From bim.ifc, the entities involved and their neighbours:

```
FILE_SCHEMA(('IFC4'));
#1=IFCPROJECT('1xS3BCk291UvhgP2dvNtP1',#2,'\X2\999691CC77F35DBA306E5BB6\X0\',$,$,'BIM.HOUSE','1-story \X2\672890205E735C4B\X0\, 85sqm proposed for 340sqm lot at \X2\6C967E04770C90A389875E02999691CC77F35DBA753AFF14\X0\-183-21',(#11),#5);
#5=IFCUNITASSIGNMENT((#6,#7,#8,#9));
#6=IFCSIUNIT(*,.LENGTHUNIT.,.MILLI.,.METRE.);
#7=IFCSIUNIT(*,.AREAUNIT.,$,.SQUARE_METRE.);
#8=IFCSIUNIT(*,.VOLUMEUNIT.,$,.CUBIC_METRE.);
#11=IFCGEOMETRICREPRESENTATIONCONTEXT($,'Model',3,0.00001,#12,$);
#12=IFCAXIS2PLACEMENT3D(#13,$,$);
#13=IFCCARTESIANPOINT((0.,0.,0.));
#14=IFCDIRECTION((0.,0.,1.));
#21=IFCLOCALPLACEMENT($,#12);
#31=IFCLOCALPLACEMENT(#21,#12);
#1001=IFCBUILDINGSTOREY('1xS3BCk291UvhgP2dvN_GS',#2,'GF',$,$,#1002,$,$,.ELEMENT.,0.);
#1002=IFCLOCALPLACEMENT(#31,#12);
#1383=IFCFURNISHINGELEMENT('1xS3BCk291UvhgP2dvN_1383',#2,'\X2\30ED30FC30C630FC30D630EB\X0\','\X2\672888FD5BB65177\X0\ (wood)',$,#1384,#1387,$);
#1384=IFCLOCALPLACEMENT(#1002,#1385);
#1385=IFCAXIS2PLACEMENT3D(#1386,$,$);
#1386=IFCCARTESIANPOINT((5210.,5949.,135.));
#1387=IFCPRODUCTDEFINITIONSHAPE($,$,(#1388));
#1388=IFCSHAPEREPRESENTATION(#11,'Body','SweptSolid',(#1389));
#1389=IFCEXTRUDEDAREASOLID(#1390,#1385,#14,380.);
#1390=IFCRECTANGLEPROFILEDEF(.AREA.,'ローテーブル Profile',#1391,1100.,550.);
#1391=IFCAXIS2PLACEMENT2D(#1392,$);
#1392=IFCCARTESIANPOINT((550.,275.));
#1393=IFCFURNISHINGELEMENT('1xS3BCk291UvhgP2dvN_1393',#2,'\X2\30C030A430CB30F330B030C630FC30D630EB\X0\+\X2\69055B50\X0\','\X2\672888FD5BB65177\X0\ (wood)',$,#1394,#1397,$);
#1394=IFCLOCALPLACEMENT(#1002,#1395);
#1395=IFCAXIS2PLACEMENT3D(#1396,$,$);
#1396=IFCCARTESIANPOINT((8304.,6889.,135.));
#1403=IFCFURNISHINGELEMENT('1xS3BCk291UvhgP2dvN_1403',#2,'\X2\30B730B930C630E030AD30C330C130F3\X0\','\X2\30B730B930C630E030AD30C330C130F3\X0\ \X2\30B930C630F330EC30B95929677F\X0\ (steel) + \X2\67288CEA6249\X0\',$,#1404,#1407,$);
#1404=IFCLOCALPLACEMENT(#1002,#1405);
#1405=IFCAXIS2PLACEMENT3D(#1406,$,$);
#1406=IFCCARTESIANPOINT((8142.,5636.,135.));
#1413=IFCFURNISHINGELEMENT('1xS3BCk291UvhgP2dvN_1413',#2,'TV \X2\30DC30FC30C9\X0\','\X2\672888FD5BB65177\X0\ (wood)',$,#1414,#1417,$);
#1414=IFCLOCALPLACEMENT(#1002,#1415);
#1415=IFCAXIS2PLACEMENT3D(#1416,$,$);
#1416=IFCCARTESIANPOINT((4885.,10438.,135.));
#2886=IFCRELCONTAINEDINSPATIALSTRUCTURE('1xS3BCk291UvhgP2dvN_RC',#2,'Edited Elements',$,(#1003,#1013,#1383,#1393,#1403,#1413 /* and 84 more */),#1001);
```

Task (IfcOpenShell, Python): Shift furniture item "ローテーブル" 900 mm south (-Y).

```python
import ifcopenshell
import ifcopenshell.api.geometry
import ifcopenshell.util.placement

model = ifcopenshell.open("bim.ifc")

item = model.by_guid("1xS3BCk291UvhgP2dvN_1383")
matrix = ifcopenshell.util.placement.get_local_placement(item.ObjectPlacement)
matrix[1, 3] -= 900.0
ifcopenshell.api.geometry.edit_object_placement(model, product=item, matrix=matrix, is_si=False)

print(ifcopenshell.util.placement.get_local_placement(item.ObjectPlacement).round(3) + 0.0)

model.write("bim_updated.ifc")
```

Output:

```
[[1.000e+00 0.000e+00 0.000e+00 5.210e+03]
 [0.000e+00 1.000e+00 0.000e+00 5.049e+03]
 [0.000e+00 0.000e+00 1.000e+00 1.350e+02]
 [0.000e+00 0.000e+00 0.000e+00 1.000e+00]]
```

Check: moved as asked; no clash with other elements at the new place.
